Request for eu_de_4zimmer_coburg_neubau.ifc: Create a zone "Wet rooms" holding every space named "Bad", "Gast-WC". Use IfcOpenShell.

First a look at what the model holds.

```python
import ifcopenshell

model = ifcopenshell.open("eu_de_4zimmer_coburg_neubau.ifc")
print(model.schema)
seen = {}
for space in model.by_type("IfcSpace"):
    seen[space.LongName] = seen.get(space.LongName, 0) + 1
for name, count in sorted(seen.items(), key=str):
    print(count, "x", name)
print("zones:", [z.Name for z in model.by_type("IfcZone")][:20])
```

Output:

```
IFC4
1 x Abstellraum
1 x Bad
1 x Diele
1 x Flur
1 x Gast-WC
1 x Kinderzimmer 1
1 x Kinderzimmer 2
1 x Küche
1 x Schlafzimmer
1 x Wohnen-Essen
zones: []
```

```python
import ifcopenshell
import ifcopenshell.api.group
import ifcopenshell.api.root

model = ifcopenshell.open("eu_de_4zimmer_coburg_neubau.ifc")

names = {"Bad", "Gast-WC"}
spaces = [s for s in model.by_type("IfcSpace") if s.LongName in names]

zone = ifcopenshell.api.root.create_entity(model, ifc_class="IfcZone", name="Wet rooms")
ifcopenshell.api.group.assign_group(model, products=spaces, group=zone)
print(len(spaces), "spaces in", zone.Name)

model.write("eu_de_4zimmer_coburg_neubau_edited.ifc")
```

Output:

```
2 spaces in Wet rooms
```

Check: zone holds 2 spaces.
